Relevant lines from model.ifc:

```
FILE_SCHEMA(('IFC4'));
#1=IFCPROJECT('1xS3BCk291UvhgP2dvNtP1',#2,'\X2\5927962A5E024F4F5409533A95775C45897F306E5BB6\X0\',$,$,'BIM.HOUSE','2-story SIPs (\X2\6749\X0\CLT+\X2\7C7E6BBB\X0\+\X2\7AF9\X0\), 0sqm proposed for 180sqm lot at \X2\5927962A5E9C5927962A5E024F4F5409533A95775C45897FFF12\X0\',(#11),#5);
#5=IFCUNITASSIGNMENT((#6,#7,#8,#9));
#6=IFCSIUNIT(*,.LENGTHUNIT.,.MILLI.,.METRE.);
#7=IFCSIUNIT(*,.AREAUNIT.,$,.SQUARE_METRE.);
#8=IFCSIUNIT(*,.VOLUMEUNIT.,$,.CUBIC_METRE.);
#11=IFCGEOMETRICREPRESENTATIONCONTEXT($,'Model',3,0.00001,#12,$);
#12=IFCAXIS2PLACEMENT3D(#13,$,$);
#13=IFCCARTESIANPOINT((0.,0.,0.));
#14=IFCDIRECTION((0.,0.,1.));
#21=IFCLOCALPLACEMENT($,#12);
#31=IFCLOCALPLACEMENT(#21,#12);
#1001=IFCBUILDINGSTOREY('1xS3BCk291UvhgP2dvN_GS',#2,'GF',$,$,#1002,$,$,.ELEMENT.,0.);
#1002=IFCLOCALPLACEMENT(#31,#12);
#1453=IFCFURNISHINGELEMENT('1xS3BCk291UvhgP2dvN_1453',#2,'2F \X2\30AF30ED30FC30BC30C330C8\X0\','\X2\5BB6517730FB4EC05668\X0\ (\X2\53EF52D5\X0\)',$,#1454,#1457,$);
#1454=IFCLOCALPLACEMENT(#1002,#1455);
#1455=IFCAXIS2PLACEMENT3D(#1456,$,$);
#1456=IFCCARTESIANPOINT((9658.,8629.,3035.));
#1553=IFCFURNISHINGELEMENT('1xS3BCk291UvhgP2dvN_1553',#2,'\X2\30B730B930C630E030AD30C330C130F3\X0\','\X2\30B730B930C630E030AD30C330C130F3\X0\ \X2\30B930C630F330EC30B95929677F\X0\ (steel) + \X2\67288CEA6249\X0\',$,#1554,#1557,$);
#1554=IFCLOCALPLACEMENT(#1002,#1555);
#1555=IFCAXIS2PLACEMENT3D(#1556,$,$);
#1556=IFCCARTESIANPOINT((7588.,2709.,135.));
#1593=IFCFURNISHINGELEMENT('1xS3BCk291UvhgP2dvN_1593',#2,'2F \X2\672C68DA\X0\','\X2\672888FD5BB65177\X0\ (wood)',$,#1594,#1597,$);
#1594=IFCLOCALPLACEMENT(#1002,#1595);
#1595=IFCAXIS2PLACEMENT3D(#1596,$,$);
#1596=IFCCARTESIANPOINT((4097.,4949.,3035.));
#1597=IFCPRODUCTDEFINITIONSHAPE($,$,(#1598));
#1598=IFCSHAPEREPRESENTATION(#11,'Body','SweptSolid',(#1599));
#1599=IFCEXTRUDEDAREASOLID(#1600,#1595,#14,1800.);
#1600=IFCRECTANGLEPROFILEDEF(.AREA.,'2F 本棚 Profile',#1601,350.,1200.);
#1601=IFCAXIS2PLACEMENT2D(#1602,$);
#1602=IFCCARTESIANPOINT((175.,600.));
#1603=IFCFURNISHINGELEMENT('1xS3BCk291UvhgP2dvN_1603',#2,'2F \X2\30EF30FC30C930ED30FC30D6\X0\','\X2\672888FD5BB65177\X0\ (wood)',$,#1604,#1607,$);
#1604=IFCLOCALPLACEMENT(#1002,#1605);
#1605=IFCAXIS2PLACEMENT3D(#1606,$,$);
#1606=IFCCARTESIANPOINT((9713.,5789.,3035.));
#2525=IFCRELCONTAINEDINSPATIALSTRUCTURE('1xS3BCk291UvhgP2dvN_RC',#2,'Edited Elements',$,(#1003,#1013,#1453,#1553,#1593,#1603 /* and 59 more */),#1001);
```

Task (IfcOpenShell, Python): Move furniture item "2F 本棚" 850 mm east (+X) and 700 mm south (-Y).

```python
import ifcopenshell
import ifcopenshell.api.geometry
import ifcopenshell.util.placement

model = ifcopenshell.open("model.ifc")

item = model.by_guid("1xS3BCk291UvhgP2dvN_1593")
matrix = ifcopenshell.util.placement.get_local_placement(item.ObjectPlacement)
matrix[0, 3] += 850.0
matrix[1, 3] -= 700.0
ifcopenshell.api.geometry.edit_object_placement(model, product=item, matrix=matrix, is_si=False)

print(ifcopenshell.util.placement.get_local_placement(item.ObjectPlacement).round(3) + 0.0)

model.write("model_updated.ifc")
```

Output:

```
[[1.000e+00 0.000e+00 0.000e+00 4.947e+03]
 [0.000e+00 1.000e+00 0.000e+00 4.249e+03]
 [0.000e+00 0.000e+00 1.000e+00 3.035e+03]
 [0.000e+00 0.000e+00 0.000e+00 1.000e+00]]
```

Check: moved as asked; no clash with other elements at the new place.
